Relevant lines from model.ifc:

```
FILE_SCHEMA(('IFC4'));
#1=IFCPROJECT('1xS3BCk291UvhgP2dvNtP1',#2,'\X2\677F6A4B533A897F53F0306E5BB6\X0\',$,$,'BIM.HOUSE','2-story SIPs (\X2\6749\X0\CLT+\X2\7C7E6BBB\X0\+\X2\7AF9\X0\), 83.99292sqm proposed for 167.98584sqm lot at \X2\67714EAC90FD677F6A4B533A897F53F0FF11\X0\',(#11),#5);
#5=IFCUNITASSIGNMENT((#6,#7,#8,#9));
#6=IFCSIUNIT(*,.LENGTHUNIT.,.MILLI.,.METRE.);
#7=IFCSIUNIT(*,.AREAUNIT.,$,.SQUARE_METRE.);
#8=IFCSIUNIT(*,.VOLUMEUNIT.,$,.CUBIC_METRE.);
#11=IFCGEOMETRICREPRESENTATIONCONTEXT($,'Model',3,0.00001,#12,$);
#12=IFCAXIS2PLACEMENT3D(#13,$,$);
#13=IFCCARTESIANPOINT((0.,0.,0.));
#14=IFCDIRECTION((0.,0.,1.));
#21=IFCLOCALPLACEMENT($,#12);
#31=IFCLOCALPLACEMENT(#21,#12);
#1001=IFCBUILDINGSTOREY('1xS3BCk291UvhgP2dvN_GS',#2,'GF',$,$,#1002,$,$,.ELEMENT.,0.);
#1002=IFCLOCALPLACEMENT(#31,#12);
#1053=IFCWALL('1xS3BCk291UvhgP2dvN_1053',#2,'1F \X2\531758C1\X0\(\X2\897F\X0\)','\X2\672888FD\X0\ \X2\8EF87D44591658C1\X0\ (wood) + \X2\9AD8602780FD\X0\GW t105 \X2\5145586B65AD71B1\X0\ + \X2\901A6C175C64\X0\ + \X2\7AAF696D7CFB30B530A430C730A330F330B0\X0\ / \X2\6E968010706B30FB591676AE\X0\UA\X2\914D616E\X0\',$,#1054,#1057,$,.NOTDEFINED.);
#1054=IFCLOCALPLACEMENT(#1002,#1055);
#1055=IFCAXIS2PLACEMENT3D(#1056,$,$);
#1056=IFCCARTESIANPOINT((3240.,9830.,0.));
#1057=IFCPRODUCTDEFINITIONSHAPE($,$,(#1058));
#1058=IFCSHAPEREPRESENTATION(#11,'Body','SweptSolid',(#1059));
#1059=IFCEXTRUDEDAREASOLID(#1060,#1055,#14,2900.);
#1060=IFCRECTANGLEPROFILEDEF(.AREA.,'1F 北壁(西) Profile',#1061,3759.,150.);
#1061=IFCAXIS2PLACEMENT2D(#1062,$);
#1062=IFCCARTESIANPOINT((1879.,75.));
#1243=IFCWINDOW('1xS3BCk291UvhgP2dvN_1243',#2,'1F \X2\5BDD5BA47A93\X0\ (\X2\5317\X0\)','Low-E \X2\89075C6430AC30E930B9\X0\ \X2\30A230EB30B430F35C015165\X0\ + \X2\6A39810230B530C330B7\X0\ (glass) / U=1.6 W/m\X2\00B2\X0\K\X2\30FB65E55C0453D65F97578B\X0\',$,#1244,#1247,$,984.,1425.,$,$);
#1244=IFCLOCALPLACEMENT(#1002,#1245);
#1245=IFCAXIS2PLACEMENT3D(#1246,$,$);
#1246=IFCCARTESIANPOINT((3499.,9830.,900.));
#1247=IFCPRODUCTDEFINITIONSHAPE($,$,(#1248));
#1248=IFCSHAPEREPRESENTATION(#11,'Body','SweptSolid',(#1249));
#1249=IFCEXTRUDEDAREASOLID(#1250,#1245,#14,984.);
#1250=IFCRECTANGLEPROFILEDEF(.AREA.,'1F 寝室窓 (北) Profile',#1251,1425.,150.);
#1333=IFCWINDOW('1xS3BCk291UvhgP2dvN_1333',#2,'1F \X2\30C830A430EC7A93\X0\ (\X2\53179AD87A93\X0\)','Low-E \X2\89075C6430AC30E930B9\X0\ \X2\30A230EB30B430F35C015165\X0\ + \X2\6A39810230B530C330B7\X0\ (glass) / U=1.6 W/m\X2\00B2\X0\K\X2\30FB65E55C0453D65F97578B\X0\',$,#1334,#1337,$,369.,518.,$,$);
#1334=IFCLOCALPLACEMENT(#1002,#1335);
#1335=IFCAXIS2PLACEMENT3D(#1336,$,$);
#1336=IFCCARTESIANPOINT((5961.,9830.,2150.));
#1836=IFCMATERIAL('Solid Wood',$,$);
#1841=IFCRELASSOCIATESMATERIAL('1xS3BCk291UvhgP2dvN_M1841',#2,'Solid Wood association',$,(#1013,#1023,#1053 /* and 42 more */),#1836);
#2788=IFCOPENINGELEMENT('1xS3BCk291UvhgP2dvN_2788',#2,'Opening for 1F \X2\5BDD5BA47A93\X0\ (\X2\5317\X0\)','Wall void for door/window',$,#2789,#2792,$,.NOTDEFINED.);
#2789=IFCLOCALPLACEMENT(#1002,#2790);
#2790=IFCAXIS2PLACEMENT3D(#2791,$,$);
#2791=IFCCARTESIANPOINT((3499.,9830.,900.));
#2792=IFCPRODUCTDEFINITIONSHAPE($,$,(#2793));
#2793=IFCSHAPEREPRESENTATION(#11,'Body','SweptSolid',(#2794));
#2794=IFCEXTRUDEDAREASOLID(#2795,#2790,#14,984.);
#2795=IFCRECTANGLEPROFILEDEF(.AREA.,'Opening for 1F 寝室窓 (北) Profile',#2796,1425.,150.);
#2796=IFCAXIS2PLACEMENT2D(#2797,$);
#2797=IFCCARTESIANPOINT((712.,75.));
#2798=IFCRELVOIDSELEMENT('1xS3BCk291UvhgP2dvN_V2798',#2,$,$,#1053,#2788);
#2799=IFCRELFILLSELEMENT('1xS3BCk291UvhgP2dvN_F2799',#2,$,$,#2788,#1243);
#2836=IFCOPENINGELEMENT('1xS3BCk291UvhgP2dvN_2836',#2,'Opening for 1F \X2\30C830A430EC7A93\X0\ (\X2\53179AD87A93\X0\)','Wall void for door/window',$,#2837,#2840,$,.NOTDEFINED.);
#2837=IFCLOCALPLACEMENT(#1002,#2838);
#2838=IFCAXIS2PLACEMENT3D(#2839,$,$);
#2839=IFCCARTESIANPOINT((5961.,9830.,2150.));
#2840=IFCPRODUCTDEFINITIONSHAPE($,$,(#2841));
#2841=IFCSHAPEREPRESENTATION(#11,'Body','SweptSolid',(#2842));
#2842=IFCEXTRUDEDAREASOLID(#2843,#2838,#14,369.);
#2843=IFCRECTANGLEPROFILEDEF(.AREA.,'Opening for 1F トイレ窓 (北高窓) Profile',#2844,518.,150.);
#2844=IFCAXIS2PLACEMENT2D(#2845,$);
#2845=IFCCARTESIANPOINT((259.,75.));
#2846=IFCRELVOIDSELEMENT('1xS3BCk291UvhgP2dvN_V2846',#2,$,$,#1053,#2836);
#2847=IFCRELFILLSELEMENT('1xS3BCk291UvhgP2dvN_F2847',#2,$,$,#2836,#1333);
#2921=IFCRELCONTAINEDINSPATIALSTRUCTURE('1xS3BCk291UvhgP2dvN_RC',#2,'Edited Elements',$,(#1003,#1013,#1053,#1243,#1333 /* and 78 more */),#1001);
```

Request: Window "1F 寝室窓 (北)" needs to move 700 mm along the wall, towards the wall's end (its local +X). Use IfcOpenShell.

```python
import ifcopenshell
import ifcopenshell.api.geometry
import ifcopenshell.util.placement

model = ifcopenshell.open("model.ifc")

window = model.by_id(1243)
opening = window.FillsVoids[0].RelatingOpeningElement
wall = opening.VoidsElements[0].RelatingBuildingElement

wall_matrix = ifcopenshell.util.placement.get_local_placement(wall.ObjectPlacement)
shift = wall_matrix[:3, 0] * 700.0
before = ifcopenshell.util.placement.get_local_placement(window.ObjectPlacement)[:3, 3].copy()

# The window is not placed relative to its opening, so move both.
for product in (opening, window):
    matrix = ifcopenshell.util.placement.get_local_placement(product.ObjectPlacement)
    matrix[:3, 3] += shift
    ifcopenshell.api.geometry.edit_object_placement(model, product=product, matrix=matrix, is_si=False)

after = ifcopenshell.util.placement.get_local_placement(window.ObjectPlacement)[:3, 3]
print("window moved by", (after - before).round(3) + 0.0)

model.write("model_updated.ifc")
```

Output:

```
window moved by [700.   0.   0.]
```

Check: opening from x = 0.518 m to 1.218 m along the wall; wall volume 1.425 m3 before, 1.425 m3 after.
